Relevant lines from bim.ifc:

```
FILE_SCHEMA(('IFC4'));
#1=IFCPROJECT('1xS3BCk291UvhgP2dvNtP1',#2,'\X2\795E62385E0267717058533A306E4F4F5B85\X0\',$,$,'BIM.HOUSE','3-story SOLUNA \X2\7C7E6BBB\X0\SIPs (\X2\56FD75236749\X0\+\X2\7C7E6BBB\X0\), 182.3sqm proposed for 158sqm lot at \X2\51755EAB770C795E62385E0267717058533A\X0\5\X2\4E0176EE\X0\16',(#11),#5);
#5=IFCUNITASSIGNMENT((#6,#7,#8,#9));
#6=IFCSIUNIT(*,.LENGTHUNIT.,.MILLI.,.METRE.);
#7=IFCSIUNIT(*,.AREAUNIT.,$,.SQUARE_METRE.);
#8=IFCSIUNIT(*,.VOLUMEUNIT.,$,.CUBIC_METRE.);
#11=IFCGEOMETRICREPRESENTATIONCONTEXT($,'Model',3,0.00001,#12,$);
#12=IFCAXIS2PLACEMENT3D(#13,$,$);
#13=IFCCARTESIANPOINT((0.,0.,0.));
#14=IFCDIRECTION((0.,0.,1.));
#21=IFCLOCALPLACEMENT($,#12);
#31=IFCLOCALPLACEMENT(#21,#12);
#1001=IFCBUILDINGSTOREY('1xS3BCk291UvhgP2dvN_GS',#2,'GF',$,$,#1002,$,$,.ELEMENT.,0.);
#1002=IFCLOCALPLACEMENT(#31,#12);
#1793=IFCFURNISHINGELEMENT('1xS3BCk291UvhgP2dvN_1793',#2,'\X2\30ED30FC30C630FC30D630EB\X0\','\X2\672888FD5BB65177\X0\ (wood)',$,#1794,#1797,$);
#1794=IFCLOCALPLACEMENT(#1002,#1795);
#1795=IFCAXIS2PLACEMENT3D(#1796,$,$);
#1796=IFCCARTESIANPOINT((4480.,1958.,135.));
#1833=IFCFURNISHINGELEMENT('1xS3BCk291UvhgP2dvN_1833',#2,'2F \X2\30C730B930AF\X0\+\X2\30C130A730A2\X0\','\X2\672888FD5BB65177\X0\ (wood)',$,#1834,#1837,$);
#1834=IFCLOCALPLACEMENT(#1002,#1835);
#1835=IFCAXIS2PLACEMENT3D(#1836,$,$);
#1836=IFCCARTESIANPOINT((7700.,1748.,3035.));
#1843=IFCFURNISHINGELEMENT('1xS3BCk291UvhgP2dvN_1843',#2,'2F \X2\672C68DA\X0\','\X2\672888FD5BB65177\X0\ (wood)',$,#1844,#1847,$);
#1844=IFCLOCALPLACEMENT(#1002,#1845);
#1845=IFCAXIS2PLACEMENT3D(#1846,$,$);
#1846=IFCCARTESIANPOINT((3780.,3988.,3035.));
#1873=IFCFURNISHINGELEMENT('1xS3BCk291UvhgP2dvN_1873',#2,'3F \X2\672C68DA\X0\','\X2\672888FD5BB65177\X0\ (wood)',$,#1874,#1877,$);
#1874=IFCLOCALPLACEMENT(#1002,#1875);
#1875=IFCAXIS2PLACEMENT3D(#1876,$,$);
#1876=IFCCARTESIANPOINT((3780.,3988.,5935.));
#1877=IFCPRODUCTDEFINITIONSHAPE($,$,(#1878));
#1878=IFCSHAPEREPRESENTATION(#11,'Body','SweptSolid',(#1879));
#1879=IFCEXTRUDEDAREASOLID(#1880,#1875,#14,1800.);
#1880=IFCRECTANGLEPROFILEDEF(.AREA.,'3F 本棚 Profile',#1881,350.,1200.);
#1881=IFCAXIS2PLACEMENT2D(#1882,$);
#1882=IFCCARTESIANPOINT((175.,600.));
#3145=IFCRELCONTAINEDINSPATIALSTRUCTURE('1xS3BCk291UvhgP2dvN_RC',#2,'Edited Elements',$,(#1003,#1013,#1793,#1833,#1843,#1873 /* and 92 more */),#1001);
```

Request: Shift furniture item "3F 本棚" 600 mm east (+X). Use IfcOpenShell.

```python
import ifcopenshell
import ifcopenshell.api.geometry
import ifcopenshell.util.placement

model = ifcopenshell.open("bim.ifc")

item = model.by_guid("1xS3BCk291UvhgP2dvN_1873")
matrix = ifcopenshell.util.placement.get_local_placement(item.ObjectPlacement)
matrix[0, 3] += 600.0
ifcopenshell.api.geometry.edit_object_placement(model, product=item, matrix=matrix, is_si=False)

print(ifcopenshell.util.placement.get_local_placement(item.ObjectPlacement).round(3) + 0.0)

model.write("bim_v2.ifc")
```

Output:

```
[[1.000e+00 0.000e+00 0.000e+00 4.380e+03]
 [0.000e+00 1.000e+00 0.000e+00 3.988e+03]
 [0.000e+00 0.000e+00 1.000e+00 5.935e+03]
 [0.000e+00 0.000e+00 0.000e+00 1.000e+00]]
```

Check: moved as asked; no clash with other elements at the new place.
